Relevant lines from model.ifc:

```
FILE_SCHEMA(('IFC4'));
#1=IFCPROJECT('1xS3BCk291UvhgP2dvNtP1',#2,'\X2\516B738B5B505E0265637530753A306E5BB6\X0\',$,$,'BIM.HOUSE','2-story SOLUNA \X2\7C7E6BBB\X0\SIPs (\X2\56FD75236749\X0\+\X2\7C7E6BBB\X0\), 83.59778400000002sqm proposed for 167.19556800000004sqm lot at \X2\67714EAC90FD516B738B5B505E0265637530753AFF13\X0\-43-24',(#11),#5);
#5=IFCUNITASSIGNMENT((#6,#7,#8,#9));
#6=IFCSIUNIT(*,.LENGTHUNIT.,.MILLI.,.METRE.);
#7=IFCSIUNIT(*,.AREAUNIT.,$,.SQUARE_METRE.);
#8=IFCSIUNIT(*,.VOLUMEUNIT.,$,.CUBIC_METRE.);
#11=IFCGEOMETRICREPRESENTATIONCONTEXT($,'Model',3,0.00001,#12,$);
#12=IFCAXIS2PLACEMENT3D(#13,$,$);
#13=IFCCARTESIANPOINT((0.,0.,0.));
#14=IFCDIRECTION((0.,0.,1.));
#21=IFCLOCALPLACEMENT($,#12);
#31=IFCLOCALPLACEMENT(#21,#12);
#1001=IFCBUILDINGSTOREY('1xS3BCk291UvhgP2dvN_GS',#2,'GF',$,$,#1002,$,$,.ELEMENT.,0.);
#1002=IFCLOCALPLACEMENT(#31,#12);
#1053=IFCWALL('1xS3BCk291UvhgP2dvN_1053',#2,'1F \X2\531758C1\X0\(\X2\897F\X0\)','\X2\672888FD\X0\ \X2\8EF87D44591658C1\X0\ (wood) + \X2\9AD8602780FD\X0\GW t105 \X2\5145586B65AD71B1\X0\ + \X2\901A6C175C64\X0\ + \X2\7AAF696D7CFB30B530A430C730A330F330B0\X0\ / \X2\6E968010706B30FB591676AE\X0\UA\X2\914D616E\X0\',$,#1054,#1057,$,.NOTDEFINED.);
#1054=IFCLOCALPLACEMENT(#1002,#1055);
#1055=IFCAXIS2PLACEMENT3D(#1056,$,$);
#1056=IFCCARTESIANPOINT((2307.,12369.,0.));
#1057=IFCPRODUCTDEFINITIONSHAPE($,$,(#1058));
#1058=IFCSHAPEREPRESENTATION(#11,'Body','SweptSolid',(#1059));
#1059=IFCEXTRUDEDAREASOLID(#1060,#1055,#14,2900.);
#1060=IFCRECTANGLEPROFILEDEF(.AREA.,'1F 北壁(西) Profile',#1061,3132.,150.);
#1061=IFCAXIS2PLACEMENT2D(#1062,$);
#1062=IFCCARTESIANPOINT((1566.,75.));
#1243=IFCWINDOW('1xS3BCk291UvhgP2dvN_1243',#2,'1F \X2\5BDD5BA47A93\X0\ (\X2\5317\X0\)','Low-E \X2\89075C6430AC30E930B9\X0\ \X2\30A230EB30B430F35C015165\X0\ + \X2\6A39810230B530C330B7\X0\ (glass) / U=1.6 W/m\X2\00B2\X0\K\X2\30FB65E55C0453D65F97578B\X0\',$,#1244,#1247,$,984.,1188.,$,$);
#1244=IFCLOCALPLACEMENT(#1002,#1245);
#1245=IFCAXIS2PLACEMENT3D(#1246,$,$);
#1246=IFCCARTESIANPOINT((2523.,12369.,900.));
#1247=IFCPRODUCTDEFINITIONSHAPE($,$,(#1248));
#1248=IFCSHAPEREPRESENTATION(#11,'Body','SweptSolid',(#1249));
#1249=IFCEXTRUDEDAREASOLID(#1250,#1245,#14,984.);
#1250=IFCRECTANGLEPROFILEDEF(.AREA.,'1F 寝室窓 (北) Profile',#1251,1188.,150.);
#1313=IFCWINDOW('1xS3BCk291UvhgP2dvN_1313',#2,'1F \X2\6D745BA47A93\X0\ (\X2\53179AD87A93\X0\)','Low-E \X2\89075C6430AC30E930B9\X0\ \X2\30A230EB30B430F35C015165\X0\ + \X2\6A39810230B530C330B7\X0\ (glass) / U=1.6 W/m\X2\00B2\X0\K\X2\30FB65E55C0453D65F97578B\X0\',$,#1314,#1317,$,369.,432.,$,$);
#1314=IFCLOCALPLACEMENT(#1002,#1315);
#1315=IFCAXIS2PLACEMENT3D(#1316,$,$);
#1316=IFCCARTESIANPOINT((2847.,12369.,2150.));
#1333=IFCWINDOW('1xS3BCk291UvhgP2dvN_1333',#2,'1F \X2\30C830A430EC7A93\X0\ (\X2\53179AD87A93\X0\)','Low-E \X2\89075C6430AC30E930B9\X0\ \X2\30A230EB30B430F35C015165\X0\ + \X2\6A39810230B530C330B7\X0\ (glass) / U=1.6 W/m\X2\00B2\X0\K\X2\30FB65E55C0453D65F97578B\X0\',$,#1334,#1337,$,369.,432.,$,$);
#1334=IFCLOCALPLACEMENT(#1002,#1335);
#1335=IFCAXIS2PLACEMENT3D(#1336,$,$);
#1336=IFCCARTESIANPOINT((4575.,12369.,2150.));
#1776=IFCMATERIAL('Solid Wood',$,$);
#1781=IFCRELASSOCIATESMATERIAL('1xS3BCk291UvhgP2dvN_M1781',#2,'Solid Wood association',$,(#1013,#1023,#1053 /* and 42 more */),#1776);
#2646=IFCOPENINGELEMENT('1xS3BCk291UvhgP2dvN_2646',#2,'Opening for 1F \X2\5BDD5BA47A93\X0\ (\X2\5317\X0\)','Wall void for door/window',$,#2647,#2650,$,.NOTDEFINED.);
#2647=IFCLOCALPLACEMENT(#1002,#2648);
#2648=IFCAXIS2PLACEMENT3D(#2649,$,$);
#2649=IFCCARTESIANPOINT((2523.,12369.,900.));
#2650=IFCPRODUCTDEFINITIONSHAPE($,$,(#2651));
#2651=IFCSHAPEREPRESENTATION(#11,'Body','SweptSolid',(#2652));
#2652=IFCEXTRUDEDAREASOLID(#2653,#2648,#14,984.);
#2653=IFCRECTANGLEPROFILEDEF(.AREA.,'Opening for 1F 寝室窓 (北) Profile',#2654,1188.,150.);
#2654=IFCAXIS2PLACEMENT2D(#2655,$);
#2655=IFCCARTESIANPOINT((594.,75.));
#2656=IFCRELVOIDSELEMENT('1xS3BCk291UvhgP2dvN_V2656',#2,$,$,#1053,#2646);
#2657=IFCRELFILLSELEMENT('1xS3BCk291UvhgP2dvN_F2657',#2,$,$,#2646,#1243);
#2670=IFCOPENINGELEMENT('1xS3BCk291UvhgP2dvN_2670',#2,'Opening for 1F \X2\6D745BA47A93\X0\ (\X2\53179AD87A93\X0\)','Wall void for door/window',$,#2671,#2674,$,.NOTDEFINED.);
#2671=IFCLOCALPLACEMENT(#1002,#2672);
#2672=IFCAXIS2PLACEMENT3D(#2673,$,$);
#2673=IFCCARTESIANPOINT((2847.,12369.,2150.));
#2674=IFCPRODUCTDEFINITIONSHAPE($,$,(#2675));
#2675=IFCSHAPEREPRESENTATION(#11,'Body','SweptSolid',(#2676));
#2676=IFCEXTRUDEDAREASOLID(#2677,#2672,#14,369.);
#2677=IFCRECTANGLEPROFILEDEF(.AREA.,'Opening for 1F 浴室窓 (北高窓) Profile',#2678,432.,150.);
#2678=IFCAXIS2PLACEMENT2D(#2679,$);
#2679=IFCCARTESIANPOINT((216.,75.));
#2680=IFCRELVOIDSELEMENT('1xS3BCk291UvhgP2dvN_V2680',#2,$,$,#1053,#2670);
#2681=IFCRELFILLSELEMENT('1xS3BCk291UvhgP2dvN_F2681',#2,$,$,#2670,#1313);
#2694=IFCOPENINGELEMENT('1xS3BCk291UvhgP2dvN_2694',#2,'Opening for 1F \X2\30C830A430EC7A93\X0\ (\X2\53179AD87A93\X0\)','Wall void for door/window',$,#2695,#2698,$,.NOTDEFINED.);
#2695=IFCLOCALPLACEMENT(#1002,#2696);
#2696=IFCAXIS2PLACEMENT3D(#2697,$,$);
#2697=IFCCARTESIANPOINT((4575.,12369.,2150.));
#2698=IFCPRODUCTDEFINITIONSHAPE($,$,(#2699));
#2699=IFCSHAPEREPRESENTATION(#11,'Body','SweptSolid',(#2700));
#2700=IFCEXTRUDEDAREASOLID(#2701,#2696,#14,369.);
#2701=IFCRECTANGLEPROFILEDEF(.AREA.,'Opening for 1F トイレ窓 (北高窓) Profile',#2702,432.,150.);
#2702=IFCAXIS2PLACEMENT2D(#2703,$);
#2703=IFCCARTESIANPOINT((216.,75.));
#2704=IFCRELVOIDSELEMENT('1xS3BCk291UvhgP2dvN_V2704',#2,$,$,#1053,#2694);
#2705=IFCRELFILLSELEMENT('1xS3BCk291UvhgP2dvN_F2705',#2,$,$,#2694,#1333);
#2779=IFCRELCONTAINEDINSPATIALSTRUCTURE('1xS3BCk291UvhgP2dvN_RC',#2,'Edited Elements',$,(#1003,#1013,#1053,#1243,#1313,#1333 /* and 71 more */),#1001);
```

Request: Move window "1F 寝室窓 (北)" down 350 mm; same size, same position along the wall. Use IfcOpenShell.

```python
import numpy as np
import ifcopenshell
import ifcopenshell.api.geometry
import ifcopenshell.util.placement
import ifcopenshell.util.unit

model = ifcopenshell.open("model.ifc")
unit_scale = ifcopenshell.util.unit.calculate_unit_scale(model)

window = model.by_id(1243)
opening = window.FillsVoids[0].RelatingOpeningElement
dz = -350.0

shift = np.array([0.0, 0.0, dz])
# The window is not placed relative to its opening, so move both.
for product in (opening, window):
    matrix = ifcopenshell.util.placement.get_local_placement(product.ObjectPlacement)
    matrix[:3, 3] += shift
    ifcopenshell.api.geometry.edit_object_placement(model, product=product, matrix=matrix, is_si=False)

print(f"moved by {dz * unit_scale:+.3f} m")

model.write("model_v2.ifc")
```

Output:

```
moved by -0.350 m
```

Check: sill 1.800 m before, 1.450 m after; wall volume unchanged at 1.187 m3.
